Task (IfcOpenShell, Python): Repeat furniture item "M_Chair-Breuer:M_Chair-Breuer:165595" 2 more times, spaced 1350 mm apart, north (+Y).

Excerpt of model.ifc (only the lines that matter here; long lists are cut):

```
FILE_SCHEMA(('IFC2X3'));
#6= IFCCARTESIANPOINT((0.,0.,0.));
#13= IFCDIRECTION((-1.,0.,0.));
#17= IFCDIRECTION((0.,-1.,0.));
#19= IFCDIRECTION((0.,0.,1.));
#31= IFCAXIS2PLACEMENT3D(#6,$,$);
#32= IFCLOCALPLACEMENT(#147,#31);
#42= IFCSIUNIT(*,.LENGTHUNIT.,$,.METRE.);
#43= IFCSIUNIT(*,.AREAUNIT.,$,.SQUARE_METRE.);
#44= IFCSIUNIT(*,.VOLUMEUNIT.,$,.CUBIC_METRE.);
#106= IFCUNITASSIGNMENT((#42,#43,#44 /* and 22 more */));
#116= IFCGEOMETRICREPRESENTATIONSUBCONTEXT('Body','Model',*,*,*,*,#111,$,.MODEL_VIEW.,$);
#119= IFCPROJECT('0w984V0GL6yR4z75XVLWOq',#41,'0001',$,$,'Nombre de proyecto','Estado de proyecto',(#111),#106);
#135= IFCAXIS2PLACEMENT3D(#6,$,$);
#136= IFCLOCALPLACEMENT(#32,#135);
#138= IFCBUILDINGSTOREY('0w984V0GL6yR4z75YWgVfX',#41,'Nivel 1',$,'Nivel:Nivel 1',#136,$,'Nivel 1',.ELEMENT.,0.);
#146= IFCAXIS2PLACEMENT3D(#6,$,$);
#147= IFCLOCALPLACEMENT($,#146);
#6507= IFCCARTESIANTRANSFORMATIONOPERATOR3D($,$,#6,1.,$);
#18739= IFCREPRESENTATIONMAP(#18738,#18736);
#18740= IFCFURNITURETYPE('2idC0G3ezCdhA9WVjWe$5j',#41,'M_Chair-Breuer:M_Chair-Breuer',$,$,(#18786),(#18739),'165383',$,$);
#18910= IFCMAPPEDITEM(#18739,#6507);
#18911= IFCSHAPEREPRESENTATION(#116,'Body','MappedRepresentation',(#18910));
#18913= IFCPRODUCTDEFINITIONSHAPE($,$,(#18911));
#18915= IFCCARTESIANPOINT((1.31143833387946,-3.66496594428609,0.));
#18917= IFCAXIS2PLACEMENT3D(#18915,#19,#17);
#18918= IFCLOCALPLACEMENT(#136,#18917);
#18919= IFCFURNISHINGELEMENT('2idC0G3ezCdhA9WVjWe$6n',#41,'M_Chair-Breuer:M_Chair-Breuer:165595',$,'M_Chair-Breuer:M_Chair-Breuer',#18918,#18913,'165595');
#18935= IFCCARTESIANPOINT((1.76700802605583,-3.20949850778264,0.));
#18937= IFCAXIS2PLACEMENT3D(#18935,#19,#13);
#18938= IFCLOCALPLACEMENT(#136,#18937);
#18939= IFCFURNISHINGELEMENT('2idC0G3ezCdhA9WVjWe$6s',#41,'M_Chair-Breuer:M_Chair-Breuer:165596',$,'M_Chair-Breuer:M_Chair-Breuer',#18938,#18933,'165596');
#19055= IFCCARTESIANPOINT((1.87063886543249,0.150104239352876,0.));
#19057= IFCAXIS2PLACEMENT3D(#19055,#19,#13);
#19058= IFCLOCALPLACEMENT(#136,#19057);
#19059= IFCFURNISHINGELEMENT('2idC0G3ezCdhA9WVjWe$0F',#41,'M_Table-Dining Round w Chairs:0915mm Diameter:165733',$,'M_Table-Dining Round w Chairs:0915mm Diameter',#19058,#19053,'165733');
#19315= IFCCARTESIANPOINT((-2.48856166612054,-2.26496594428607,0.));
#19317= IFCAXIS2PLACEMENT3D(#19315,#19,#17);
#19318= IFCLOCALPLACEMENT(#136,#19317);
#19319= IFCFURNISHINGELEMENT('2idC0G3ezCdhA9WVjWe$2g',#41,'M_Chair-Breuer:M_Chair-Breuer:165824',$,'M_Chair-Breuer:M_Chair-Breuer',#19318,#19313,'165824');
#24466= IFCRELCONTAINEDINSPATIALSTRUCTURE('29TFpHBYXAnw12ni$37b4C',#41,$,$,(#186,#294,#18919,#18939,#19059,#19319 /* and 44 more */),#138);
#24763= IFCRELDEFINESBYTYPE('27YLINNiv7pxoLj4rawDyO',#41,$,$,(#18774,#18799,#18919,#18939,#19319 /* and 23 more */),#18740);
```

```python
import numpy as np
import ifcopenshell
import ifcopenshell.api.geometry
import ifcopenshell.api.root
import ifcopenshell.util.element
import ifcopenshell.util.placement

model = ifcopenshell.open("model.ifc")


def reuse_history(source, copy):
    """copy_class also copies each property set's owner history, people and application; keep the originals."""
    for rel in copy.IsDefinedBy:
        if rel.is_a("IfcRelDefinesByProperties") and (history := rel.RelatingPropertyDefinition.OwnerHistory):
            rel.RelatingPropertyDefinition.OwnerHistory = source.OwnerHistory
            ifcopenshell.util.element.remove_deep2(model, history)


source = model.by_id(18919)
base = ifcopenshell.util.placement.get_local_placement(source.ObjectPlacement)
step = np.array([0.0, 1.0, 0.0]) * 1.35

for i in range(1, 3):
    copy = ifcopenshell.api.root.copy_class(model, product=source)
    copy.Representation = ifcopenshell.util.element.copy_deep(
        model, source.Representation, exclude=["IfcGeometricRepresentationContext", "IfcRepresentationMap"]
    )
    copy.Name = "M_Chair-Breuer:M_Chair-Breuer"
    copy.Tag = None
    reuse_history(source, copy)
    matrix = base.copy()
    matrix[:3, 3] += i * step
    print("added at", matrix[:3, 3].round(3) + 0.0)
    ifcopenshell.api.geometry.edit_object_placement(model, product=copy, matrix=matrix, is_si=False)

model.write("model_v2.ifc")
```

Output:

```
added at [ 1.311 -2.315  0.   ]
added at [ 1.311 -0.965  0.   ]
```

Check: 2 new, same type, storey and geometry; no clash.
